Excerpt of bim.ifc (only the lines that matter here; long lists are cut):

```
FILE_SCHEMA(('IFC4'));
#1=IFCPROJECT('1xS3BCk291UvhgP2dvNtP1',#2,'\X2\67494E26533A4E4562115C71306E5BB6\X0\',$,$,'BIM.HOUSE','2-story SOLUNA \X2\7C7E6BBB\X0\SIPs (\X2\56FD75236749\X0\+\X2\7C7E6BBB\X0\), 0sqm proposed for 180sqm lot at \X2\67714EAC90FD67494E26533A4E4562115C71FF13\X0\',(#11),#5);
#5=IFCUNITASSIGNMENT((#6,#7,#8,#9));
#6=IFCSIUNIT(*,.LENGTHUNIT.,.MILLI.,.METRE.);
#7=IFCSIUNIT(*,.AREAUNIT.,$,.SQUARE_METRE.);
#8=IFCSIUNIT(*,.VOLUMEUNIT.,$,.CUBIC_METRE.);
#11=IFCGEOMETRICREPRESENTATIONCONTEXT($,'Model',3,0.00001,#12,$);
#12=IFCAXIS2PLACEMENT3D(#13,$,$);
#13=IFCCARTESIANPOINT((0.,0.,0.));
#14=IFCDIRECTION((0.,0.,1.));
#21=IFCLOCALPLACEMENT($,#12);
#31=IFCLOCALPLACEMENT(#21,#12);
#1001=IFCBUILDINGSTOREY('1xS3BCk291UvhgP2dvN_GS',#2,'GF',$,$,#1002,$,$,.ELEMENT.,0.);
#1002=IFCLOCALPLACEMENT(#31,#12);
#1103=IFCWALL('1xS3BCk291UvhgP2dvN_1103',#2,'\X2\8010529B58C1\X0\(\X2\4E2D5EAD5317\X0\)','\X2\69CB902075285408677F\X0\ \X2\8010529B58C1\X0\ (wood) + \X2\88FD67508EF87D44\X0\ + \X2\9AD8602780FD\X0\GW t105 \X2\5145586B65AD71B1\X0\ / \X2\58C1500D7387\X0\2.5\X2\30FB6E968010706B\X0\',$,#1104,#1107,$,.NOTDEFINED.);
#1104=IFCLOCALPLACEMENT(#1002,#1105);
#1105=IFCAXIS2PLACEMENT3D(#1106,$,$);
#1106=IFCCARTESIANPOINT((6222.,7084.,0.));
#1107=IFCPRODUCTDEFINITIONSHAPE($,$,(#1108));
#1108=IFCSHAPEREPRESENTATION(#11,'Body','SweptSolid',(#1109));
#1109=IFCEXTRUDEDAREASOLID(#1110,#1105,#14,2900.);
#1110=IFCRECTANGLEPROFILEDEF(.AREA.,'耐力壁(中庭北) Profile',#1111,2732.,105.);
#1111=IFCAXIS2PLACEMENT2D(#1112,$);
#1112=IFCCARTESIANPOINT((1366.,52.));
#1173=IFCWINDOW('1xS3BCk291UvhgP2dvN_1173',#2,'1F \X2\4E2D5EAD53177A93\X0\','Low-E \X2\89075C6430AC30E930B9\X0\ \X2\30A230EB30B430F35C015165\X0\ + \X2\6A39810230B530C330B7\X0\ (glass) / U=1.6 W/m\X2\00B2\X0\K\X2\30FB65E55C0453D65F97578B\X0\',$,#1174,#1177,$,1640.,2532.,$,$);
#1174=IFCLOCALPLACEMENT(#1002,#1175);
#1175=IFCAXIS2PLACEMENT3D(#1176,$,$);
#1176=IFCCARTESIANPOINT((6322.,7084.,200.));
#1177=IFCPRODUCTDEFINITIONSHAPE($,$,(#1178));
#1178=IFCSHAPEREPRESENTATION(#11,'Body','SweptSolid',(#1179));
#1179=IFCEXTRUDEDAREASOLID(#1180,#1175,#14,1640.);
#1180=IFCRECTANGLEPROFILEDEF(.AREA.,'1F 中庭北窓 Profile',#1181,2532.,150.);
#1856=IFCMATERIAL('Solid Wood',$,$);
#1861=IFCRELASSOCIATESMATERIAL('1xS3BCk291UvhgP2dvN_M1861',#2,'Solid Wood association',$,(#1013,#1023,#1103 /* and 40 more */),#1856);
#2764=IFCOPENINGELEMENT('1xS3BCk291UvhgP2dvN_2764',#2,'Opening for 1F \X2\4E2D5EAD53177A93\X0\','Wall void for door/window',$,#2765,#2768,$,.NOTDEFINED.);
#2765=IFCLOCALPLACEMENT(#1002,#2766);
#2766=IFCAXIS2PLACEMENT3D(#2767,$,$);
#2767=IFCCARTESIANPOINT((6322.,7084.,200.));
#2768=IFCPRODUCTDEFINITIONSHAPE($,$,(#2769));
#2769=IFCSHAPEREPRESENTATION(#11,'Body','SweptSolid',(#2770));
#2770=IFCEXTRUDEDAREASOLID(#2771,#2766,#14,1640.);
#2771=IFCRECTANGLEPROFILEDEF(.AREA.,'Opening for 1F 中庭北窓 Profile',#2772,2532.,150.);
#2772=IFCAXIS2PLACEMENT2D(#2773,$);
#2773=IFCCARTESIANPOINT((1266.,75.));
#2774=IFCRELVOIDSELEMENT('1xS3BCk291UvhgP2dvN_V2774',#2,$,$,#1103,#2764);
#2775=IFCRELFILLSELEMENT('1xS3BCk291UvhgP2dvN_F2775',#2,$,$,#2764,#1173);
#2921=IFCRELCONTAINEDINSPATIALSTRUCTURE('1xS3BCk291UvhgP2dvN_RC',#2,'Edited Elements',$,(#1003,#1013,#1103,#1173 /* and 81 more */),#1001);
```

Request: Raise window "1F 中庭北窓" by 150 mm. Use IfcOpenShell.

```python
import numpy as np
import ifcopenshell
import ifcopenshell.api.geometry
import ifcopenshell.util.placement
import ifcopenshell.util.unit

model = ifcopenshell.open("bim.ifc")
unit_scale = ifcopenshell.util.unit.calculate_unit_scale(model)

window = model.by_guid("1xS3BCk291UvhgP2dvN_1173")
opening = window.FillsVoids[0].RelatingOpeningElement
dz = 0.15 / unit_scale

shift = np.array([0.0, 0.0, dz])
# The window is not placed relative to its opening, so move both.
for product in (opening, window):
    matrix = ifcopenshell.util.placement.get_local_placement(product.ObjectPlacement)
    matrix[:3, 3] += shift
    ifcopenshell.api.geometry.edit_object_placement(model, product=product, matrix=matrix, is_si=False)

print(f"moved by {dz * unit_scale:+.3f} m")

model.write("bim-out.ifc")
```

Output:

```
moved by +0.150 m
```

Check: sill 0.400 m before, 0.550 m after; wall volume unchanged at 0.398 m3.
